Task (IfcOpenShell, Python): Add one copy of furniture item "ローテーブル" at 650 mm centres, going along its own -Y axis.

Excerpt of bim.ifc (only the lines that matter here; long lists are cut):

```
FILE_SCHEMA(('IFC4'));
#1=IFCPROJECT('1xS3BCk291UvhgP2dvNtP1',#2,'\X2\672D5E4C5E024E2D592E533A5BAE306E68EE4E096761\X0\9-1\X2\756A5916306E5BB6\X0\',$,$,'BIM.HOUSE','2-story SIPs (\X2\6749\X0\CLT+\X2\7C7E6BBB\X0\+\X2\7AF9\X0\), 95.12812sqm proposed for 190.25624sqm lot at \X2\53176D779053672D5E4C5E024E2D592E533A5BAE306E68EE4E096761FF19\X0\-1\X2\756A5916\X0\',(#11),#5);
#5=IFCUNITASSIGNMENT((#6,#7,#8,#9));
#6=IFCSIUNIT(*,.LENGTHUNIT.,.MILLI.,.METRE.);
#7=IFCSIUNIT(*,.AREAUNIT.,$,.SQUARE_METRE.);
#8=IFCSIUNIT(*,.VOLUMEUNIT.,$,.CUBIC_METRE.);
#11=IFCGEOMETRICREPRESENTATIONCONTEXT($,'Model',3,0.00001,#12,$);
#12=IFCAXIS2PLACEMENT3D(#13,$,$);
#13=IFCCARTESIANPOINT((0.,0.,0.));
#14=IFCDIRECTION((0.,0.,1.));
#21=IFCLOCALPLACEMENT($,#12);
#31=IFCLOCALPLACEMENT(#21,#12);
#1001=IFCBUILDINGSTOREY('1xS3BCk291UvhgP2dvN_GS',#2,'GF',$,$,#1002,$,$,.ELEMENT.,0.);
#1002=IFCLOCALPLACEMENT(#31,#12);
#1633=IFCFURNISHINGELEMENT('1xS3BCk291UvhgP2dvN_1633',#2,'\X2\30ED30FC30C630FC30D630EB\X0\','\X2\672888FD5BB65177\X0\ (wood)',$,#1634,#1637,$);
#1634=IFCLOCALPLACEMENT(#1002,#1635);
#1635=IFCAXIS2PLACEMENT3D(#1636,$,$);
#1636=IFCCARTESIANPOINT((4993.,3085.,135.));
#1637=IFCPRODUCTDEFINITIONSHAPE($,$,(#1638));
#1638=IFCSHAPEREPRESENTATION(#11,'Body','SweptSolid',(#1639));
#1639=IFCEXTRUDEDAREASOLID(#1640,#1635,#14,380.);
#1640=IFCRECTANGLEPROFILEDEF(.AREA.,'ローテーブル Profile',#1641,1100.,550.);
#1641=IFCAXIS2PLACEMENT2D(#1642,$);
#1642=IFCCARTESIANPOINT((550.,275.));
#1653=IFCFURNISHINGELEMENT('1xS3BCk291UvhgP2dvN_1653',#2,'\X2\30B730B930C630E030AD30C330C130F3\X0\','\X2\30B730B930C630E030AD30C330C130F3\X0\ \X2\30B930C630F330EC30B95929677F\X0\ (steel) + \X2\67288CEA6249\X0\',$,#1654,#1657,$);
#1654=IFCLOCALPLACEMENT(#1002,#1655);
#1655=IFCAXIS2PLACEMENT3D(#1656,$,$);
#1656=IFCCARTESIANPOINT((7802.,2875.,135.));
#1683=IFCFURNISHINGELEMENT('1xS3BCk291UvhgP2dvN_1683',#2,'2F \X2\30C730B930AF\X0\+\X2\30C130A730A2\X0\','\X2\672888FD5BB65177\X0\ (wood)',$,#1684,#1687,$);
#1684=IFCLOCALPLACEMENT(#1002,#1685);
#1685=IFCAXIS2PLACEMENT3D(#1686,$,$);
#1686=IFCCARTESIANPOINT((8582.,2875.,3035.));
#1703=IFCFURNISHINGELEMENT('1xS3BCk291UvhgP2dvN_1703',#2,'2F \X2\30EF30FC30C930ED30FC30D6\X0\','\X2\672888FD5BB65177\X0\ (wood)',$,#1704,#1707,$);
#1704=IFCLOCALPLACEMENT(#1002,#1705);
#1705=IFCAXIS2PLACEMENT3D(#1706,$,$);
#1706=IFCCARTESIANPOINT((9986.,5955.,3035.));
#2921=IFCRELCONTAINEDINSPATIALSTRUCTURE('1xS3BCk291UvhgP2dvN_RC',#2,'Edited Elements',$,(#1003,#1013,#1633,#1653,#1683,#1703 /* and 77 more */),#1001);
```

```python
import ifcopenshell
import ifcopenshell.api.geometry
import ifcopenshell.api.root
import ifcopenshell.util.element
import ifcopenshell.util.placement
import ifcopenshell.util.unit

model = ifcopenshell.open("bim.ifc")
unit_scale = ifcopenshell.util.unit.calculate_unit_scale(model)


def reuse_history(source, copy):
    """copy_class also copies each property set's owner history, people and application; keep the originals."""
    for rel in copy.IsDefinedBy:
        if rel.is_a("IfcRelDefinesByProperties") and (history := rel.RelatingPropertyDefinition.OwnerHistory):
            rel.RelatingPropertyDefinition.OwnerHistory = source.OwnerHistory
            ifcopenshell.util.element.remove_deep2(model, history)


source = model.by_guid("1xS3BCk291UvhgP2dvN_1633")
base = ifcopenshell.util.placement.get_local_placement(source.ObjectPlacement)
step = -base[:3, 1] * 0.65 / unit_scale

for i in range(1, 2):
    copy = ifcopenshell.api.root.copy_class(model, product=source)
    copy.Representation = ifcopenshell.util.element.copy_deep(
        model, source.Representation, exclude=["IfcGeometricRepresentationContext", "IfcRepresentationMap"]
    )
    reuse_history(source, copy)
    matrix = base.copy()
    matrix[:3, 3] += i * step
    print("added at", matrix[:3, 3].round(3) + 0.0)
    ifcopenshell.api.geometry.edit_object_placement(model, product=copy, matrix=matrix, is_si=False)

model.write("bim-out.ifc")
```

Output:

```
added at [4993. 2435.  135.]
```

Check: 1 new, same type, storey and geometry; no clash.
